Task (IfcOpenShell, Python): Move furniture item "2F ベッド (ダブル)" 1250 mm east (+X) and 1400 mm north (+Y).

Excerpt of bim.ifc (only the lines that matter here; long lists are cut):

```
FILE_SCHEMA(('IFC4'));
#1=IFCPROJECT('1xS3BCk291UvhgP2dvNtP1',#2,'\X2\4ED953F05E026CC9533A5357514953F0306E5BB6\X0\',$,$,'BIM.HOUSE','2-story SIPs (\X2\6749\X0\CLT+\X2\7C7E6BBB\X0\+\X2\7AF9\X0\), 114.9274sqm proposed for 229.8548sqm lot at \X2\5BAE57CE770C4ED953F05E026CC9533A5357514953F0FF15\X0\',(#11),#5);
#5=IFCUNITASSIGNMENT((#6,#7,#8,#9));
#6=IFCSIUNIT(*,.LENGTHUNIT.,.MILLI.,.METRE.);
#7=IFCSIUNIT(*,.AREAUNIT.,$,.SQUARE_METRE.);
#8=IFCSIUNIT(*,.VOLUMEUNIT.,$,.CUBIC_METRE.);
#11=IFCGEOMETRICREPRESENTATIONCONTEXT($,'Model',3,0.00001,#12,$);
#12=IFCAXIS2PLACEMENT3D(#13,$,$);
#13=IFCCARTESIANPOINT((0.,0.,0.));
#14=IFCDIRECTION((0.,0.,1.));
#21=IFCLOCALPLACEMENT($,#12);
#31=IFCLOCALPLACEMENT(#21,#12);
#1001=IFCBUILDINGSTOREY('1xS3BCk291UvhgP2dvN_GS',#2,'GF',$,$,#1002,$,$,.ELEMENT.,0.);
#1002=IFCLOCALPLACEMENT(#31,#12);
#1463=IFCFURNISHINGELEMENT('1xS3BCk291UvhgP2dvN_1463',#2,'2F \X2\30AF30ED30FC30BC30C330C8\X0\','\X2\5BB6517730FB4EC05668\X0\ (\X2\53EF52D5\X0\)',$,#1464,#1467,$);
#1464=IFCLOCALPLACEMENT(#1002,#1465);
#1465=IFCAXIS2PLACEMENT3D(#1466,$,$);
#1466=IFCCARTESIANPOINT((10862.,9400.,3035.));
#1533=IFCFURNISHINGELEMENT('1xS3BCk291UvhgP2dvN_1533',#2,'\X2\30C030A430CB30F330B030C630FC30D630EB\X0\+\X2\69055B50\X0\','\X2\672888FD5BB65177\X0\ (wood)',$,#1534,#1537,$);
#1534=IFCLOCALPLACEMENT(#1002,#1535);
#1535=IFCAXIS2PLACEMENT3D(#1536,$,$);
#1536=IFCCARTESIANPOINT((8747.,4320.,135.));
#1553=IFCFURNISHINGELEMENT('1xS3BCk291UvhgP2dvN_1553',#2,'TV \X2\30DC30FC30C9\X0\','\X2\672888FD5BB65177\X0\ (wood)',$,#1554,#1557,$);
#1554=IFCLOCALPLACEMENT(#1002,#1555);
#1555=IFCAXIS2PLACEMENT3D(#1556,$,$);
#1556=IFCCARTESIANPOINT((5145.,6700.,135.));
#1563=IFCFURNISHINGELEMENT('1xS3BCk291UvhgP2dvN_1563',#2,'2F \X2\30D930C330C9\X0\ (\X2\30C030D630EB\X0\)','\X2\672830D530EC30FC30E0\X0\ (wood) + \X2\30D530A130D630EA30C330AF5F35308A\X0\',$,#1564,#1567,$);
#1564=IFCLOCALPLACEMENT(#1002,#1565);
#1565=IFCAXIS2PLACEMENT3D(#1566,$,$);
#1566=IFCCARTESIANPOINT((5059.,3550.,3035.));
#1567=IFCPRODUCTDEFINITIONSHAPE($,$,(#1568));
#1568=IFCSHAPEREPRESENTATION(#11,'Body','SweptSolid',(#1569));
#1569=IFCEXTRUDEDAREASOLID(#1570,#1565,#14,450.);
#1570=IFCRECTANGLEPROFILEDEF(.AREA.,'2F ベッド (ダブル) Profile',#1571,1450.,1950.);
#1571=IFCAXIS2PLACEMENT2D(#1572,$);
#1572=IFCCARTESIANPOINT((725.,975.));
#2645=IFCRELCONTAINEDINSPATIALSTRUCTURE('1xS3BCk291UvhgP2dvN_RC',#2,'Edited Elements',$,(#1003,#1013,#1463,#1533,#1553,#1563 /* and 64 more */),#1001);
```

```python
import ifcopenshell
import ifcopenshell.api.geometry
import ifcopenshell.util.placement
import ifcopenshell.util.unit

model = ifcopenshell.open("bim.ifc")
unit_scale = ifcopenshell.util.unit.calculate_unit_scale(model)

item = model.by_guid("1xS3BCk291UvhgP2dvN_1563")
matrix = ifcopenshell.util.placement.get_local_placement(item.ObjectPlacement)
matrix[0, 3] += 1.25 / unit_scale
matrix[1, 3] += 1.4 / unit_scale
ifcopenshell.api.geometry.edit_object_placement(model, product=item, matrix=matrix, is_si=False)

print(ifcopenshell.util.placement.get_local_placement(item.ObjectPlacement).round(3) + 0.0)

model.write("bim_edited.ifc")
```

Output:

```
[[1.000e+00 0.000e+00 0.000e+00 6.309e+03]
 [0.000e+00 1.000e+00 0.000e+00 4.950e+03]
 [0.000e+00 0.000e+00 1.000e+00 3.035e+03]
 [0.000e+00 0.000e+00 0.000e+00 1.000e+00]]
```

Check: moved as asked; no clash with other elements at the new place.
